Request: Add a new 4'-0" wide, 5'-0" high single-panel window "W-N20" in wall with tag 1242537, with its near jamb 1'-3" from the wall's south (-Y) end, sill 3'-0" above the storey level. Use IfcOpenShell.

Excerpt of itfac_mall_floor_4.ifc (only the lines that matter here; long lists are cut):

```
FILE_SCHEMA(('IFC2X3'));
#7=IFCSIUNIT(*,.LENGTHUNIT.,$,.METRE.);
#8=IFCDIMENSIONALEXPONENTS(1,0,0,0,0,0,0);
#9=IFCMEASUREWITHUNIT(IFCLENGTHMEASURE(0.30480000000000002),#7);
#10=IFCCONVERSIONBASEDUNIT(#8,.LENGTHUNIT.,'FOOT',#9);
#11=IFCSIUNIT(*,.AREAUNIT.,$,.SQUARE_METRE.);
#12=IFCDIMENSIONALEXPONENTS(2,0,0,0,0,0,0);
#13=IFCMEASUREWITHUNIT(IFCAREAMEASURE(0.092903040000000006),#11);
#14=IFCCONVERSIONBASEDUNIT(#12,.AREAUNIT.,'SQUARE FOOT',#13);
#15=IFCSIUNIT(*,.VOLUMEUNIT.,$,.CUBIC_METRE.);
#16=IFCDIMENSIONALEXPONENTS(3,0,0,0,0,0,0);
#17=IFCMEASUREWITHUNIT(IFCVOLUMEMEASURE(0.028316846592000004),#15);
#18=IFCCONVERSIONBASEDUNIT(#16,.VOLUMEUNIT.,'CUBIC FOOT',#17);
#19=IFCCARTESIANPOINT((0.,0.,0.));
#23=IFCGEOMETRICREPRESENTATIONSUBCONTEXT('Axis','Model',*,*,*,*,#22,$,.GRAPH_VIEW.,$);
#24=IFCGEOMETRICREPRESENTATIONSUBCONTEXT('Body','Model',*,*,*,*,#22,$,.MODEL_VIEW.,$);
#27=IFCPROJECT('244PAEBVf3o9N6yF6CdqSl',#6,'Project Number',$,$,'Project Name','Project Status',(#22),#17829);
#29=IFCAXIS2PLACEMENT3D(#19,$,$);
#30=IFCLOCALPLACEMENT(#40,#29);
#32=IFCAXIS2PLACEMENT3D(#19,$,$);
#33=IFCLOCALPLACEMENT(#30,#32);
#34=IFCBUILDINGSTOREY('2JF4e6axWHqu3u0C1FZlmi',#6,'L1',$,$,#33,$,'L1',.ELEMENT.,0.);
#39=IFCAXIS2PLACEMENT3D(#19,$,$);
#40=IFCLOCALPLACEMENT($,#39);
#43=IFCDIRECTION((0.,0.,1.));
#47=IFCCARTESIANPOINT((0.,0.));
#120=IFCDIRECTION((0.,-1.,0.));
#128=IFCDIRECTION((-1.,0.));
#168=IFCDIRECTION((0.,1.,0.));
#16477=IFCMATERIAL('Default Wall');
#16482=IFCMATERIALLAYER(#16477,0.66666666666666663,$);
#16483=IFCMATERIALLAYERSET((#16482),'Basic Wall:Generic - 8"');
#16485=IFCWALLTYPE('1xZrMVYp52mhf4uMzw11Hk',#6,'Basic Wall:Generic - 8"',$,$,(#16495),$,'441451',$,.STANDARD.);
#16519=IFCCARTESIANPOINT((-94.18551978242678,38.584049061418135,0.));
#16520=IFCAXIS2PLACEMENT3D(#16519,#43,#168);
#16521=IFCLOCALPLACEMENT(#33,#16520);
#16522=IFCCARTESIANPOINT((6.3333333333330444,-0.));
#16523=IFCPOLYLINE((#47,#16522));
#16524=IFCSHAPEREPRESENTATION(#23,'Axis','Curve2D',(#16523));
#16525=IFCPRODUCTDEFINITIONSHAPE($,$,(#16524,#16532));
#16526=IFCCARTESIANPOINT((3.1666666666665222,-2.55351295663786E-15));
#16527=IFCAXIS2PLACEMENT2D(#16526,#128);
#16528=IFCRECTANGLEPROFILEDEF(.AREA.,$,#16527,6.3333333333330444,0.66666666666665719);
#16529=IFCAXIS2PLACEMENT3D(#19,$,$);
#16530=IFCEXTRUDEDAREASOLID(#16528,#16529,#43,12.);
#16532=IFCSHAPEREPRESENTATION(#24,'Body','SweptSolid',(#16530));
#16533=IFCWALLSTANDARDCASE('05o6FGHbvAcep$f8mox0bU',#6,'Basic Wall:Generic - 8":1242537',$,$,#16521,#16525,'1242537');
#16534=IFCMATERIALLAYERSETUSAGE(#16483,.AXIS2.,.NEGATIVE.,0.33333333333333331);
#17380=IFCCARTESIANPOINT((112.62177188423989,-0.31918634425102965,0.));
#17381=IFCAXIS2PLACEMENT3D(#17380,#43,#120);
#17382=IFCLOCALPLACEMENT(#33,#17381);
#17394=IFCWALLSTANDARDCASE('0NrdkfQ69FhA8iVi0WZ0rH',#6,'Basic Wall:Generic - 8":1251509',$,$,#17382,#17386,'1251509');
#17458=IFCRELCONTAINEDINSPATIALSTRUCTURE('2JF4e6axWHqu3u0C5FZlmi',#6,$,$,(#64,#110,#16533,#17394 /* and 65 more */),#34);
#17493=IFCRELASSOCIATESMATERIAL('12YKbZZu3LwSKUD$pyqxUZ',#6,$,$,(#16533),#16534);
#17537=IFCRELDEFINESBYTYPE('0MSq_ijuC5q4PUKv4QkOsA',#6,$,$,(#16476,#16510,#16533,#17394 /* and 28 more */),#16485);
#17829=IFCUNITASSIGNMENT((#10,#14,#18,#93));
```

```python
import numpy as np
import ifcopenshell
import ifcopenshell.api.feature
import ifcopenshell.api.geometry
import ifcopenshell.api.root
import ifcopenshell.api.spatial
import ifcopenshell.api.type
import ifcopenshell.geom
import ifcopenshell.util.element
import ifcopenshell.util.placement
import ifcopenshell.util.representation
import ifcopenshell.util.shape
import ifcopenshell.util.unit

model = ifcopenshell.open("itfac_mall_floor_4.ifc")
unit_scale = ifcopenshell.util.unit.calculate_unit_scale(model)
settings = ifcopenshell.geom.settings()


def volume(element):
    """Net volume in cubic metres, openings subtracted."""
    shape = ifcopenshell.geom.create_shape(settings, element)
    return ifcopenshell.util.shape.get_volume(shape.geometry)


wall = model.by_guid("05o6FGHbvAcep$f8mox0bU")
storey = ifcopenshell.util.element.get_container(wall, ifc_class="IfcBuildingStorey")
context = ifcopenshell.util.representation.get_context(model, "Model", "Body", "MODEL_VIEW")
before = volume(wall)

width, height, from_end, sill = 1.2192, 1.524, 0.381, 0.9144  # metres

# The wall runs along its own X axis, and the end named is its -X end.
wall_shape = ifcopenshell.geom.create_shape(settings, wall)
x, y, z = ifcopenshell.util.shape.get_vertices(wall_shape.geometry).T
start = x.min() + from_end
face, thickness = float(y.min()), float(y.max() - y.min())
wall_matrix = ifcopenshell.util.placement.get_local_placement(wall.ObjectPlacement)
level = ifcopenshell.util.placement.get_local_placement(storey.ObjectPlacement)[2, 3]


def in_wall(x, y):
    """Placement at x, y metres in the wall's axes, at sill height."""
    matrix = wall_matrix.copy()
    matrix[:, 3] = wall_matrix @ np.array([x / unit_scale, y / unit_scale, 0.0, 1.0])
    matrix[2, 3] = level + sill / unit_scale
    return matrix


# Opening: a box that overshoots both wall faces by 50 mm.
opening = ifcopenshell.api.root.create_entity(model, ifc_class="IfcOpeningElement")
box = ifcopenshell.api.geometry.add_wall_representation(
    model, context=context, length=width, height=height, thickness=thickness + 0.1
)
ifcopenshell.api.geometry.assign_representation(model, product=opening, representation=box)
ifcopenshell.api.geometry.edit_object_placement(model, product=opening, matrix=in_wall(start, face - 0.05), is_si=False)
ifcopenshell.api.feature.add_feature(model, feature=opening, element=wall)

window = ifcopenshell.api.root.create_entity(model, ifc_class="IfcWindow", name="W-N20")
window.OverallWidth, window.OverallHeight = width / unit_scale, height / unit_scale
body = ifcopenshell.api.geometry.add_window_representation(
    model,
    context=context,
    overall_width=window.OverallWidth,
    overall_height=window.OverallHeight,
    partition_type="SINGLE_PANEL",
)
ifcopenshell.api.geometry.assign_representation(model, product=window, representation=body)
ifcopenshell.api.spatial.assign_container(model, products=[window], relating_structure=storey)
fills = ifcopenshell.api.feature.add_filling(model, opening=opening, element=window)
fills.OwnerHistory = window.OwnerHistory  # required in IFC2X3

# IFC2X3 keeps the operation on the window style.
style = ifcopenshell.api.root.create_entity(model, ifc_class="IfcWindowStyle", name="W-N20")
style.OperationType, style.ConstructionType = "SINGLE_PANEL", "NOTDEFINED"
style.ParameterTakesPrecedence = style.Sizeable = False
ifcopenshell.api.type.assign_type(model, related_objects=[window], relating_type=style)

# Centre the window in the wall's thickness.
ifcopenshell.api.geometry.edit_object_placement(model, product=window, matrix=in_wall(start, face), is_si=False)
window_shape = ifcopenshell.geom.create_shape(settings, window)
depth = ifcopenshell.util.shape.get_vertices(window_shape.geometry)[:, 1]
offset = face + thickness / 2 - (depth.min() + depth.max()) / 2
ifcopenshell.api.geometry.edit_object_placement(model, product=window, matrix=in_wall(start, offset), is_si=False)

after = volume(wall)

print(f"wall volume {before:.3f} -> {after:.3f} m3")

model.write("itfac_mall_floor_4-out.ifc")
```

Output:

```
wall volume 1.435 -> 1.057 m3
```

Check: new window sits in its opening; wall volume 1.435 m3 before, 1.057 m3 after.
